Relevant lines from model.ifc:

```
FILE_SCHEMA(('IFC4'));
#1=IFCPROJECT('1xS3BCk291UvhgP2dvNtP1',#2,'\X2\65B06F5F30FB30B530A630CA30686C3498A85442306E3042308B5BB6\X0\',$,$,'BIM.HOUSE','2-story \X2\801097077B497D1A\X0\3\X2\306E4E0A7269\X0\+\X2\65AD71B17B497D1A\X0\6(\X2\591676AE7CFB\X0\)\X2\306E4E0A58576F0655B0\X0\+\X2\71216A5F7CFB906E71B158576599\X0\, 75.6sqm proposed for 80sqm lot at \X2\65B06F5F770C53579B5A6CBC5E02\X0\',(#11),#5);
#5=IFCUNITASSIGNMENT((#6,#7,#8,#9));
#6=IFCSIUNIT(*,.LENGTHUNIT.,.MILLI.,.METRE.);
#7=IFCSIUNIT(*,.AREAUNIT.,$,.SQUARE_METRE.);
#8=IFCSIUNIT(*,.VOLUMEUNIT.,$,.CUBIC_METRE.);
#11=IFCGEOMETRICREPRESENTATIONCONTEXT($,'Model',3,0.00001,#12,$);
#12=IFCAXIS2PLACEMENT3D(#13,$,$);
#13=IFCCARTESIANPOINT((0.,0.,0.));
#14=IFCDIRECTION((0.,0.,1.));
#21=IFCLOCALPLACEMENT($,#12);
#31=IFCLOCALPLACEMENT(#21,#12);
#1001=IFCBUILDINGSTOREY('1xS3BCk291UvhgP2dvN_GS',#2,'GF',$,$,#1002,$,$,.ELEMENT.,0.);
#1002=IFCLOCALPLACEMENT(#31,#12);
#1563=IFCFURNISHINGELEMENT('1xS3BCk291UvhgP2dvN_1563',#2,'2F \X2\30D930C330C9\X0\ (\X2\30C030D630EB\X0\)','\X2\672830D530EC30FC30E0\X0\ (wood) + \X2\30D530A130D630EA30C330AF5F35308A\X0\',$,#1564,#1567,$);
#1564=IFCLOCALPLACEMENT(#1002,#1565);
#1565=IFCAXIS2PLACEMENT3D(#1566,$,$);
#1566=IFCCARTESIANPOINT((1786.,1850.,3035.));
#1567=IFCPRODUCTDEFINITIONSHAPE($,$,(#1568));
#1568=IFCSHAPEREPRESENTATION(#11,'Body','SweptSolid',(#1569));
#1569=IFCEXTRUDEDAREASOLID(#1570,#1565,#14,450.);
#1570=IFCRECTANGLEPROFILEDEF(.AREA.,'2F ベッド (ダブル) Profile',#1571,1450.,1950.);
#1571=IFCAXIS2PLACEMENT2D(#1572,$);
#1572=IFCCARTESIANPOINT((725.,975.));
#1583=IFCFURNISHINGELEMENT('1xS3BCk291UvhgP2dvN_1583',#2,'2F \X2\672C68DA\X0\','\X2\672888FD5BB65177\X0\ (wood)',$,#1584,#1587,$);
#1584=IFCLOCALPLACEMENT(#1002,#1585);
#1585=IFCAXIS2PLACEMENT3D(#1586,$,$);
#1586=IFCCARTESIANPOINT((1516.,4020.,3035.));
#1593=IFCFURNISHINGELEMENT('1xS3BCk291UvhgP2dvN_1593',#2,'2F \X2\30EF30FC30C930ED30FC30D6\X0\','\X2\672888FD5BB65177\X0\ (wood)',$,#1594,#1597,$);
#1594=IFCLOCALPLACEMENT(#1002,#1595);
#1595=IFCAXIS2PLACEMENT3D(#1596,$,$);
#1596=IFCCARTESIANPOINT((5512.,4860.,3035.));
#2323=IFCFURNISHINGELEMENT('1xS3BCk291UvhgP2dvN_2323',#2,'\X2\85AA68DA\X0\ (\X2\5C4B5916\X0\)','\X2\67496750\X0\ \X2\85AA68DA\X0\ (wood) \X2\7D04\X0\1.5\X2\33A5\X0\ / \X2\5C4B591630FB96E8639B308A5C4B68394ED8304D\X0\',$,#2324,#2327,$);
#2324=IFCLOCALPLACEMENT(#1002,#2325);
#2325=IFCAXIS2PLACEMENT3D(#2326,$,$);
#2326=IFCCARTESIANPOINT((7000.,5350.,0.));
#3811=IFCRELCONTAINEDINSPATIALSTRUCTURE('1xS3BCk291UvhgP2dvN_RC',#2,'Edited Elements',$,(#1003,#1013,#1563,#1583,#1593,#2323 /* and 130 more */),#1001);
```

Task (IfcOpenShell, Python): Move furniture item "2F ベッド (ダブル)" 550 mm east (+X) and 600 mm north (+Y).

```python
import ifcopenshell
import ifcopenshell.api.geometry
import ifcopenshell.util.placement

model = ifcopenshell.open("model.ifc")

item = model.by_guid("1xS3BCk291UvhgP2dvN_1563")
matrix = ifcopenshell.util.placement.get_local_placement(item.ObjectPlacement)
matrix[0, 3] += 550.0
matrix[1, 3] += 600.0
ifcopenshell.api.geometry.edit_object_placement(model, product=item, matrix=matrix, is_si=False)

print(ifcopenshell.util.placement.get_local_placement(item.ObjectPlacement).round(3) + 0.0)

model.write("model_rev.ifc")
```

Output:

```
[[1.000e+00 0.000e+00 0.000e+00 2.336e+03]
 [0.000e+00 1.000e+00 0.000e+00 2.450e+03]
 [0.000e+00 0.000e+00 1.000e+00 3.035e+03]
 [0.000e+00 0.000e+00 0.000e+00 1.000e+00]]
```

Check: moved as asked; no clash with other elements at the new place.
